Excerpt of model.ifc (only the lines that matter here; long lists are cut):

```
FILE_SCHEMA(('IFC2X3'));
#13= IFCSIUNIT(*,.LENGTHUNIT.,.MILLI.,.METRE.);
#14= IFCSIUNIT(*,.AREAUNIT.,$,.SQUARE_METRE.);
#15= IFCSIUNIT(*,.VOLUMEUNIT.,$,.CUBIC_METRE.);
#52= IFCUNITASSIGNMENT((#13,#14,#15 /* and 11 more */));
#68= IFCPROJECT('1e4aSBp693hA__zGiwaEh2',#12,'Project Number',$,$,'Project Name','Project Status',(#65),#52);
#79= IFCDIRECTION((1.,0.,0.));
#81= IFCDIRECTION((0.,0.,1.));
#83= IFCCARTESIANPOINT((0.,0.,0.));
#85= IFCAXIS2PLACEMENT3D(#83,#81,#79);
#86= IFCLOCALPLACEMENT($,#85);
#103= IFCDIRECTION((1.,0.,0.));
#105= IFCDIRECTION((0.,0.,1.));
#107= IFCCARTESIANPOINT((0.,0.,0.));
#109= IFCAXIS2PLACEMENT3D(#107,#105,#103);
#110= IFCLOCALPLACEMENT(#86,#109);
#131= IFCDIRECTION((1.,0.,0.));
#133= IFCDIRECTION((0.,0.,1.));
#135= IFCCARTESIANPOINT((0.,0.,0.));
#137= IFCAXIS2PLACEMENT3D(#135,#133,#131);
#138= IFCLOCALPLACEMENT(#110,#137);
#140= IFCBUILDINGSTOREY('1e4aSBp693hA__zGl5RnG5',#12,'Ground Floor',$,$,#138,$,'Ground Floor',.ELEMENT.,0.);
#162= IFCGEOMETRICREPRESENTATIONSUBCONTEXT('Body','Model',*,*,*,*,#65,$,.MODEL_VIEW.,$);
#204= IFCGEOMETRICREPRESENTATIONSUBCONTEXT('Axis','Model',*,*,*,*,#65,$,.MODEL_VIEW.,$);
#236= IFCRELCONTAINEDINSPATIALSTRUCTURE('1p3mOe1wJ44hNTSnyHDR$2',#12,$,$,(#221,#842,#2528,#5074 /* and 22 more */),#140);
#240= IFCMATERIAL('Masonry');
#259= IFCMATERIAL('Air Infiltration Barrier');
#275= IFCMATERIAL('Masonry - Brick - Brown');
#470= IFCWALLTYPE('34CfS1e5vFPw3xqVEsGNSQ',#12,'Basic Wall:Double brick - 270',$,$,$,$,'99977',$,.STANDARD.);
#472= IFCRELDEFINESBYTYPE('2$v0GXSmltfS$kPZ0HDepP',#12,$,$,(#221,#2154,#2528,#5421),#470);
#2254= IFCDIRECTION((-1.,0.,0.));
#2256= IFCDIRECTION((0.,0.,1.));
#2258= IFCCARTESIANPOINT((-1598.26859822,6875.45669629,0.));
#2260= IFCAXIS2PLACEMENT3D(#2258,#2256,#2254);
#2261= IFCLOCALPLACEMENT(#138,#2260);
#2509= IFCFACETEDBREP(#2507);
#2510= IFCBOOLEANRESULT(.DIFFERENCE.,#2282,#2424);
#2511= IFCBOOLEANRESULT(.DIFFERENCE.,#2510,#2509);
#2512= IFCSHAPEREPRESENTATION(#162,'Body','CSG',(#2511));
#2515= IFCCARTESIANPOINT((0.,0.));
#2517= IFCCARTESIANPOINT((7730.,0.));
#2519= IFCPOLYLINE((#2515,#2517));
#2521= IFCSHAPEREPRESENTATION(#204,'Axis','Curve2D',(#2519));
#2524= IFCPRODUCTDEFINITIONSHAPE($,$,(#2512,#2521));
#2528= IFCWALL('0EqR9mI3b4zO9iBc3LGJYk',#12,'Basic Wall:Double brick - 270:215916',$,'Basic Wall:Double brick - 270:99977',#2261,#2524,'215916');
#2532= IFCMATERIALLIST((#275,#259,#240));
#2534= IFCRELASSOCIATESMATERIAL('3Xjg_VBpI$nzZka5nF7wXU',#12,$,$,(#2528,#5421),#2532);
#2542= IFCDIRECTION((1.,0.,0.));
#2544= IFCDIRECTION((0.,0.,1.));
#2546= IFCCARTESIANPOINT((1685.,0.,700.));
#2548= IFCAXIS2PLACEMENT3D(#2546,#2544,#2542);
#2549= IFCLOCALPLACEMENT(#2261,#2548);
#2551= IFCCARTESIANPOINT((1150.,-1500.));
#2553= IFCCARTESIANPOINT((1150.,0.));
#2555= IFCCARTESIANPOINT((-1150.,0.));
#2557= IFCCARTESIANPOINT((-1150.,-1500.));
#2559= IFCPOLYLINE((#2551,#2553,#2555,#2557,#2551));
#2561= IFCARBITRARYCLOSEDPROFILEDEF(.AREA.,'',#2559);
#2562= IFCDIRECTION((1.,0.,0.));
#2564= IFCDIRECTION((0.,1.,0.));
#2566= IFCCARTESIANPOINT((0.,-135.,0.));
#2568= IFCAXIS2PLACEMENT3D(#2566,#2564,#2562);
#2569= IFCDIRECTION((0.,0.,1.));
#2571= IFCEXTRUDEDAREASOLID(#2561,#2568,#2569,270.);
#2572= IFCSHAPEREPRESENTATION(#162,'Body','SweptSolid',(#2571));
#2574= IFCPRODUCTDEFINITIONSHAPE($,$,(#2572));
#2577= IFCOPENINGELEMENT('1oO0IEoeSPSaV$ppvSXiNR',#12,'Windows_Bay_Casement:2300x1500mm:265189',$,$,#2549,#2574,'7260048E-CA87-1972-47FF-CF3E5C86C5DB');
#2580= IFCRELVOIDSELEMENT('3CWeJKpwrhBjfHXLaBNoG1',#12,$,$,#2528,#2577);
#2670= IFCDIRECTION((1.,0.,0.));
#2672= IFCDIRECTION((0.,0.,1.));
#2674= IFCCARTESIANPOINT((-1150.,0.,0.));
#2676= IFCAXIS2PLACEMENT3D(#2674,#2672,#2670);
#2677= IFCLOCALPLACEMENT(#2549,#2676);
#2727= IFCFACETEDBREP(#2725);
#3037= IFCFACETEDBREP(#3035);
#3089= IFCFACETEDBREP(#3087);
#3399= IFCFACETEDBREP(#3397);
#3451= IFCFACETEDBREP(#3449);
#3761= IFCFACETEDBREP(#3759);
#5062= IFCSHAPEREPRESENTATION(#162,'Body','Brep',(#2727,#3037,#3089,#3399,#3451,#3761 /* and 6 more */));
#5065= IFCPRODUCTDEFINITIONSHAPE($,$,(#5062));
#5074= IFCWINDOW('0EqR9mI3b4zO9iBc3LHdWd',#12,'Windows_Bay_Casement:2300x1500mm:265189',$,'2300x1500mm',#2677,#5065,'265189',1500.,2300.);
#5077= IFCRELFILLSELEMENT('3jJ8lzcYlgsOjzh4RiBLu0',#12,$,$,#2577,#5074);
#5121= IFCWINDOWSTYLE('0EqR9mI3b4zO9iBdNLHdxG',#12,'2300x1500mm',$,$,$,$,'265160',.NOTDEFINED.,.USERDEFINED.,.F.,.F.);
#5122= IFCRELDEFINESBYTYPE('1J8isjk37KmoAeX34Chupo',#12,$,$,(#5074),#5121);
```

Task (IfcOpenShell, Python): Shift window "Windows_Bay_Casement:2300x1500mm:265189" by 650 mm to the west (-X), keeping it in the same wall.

```python
import ifcopenshell
import ifcopenshell.api.geometry
import ifcopenshell.util.placement
import ifcopenshell.util.unit

model = ifcopenshell.open("model.ifc")
unit_scale = ifcopenshell.util.unit.calculate_unit_scale(model)

window = model.by_id(5074)
opening = window.FillsVoids[0].RelatingOpeningElement
wall = opening.VoidsElements[0].RelatingBuildingElement

wall_matrix = ifcopenshell.util.placement.get_local_placement(wall.ObjectPlacement)
shift = wall_matrix[:3, 0] * 0.65 / unit_scale
before = ifcopenshell.util.placement.get_local_placement(window.ObjectPlacement)[:3, 3].copy()

# The window is placed relative to its opening, so it follows when the opening moves.
matrix = ifcopenshell.util.placement.get_local_placement(opening.ObjectPlacement)
matrix[:3, 3] += shift
ifcopenshell.api.geometry.edit_object_placement(
    model, product=opening, matrix=matrix, is_si=False, should_transform_children=True
)

after = ifcopenshell.util.placement.get_local_placement(window.ObjectPlacement)[:3, 3]
print("window moved by", (after - before).round(3) + 0.0)

model.write("model_v2.ifc")
```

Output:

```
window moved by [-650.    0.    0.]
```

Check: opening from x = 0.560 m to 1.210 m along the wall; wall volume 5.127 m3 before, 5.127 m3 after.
